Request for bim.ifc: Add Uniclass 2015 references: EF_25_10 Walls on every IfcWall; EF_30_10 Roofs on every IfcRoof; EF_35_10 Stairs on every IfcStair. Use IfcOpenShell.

First a look at what the model holds.

```python
import ifcopenshell

model = ifcopenshell.open("bim.ifc")
print(model.schema)
print("classifications:", [c.Name for c in model.by_type("IfcClassification")])
for ifc_class in ("IfcDoor", "IfcRoof", "IfcStair", "IfcWall", "IfcWindow"):
    print(ifc_class, len(model.by_type(ifc_class)))
```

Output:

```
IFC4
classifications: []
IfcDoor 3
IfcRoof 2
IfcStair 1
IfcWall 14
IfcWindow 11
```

```python
import ifcopenshell
import ifcopenshell.api.classification

model = ifcopenshell.open("bim.ifc")

system = ifcopenshell.api.classification.add_classification(model, classification="Uniclass 2015")

codes = {
    "IfcWall": ("EF_25_10", "Walls"),
    "IfcRoof": ("EF_30_10", "Roofs"),
    "IfcStair": ("EF_35_10", "Stairs"),
}
for ifc_class, (code, name) in codes.items():
    products = model.by_type(ifc_class)
    ifcopenshell.api.classification.add_reference(
        model, products=products, classification=system, identification=code, name=name
    )
    print(code, len(products))

model.write("bim-out.ifc")
```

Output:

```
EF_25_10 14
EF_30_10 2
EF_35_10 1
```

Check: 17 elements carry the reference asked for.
